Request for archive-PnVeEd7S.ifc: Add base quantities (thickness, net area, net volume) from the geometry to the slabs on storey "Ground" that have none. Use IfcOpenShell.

First a look at what the model holds.

```python
import ifcopenshell
import ifcopenshell.util.element
import ifcopenshell.util.unit

model = ifcopenshell.open("archive-PnVeEd7S.ifc")
print(model.schema)
for unit_type in ("LENGTHUNIT", "AREAUNIT", "VOLUMEUNIT"):
    print(unit_type, ifcopenshell.util.unit.calculate_unit_scale(model, unit_type))
storey = next(s for s in model.by_type("IfcBuildingStorey") if s.Name == "Ground")
slabs = [e for e in ifcopenshell.util.element.get_decomposition(storey) if e.is_a("IfcSlab")]
for e in sorted(slabs, key=lambda e: e.id()):
    print(e.id(), e.is_a(), e.Name, list(ifcopenshell.util.element.get_psets(e, qtos_only=True)), sep=" | ")
```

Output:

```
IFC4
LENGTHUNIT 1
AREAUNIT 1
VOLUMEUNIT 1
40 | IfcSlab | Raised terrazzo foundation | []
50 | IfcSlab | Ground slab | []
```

```python
import ifcopenshell
import ifcopenshell.api.pset
import ifcopenshell.geom
import ifcopenshell.util.element
import ifcopenshell.util.shape
import ifcopenshell.util.unit

model = ifcopenshell.open("archive-PnVeEd7S.ifc")
unit_scale = ifcopenshell.util.unit.calculate_unit_scale(model)
area_scale = ifcopenshell.util.unit.calculate_unit_scale(model, "AREAUNIT")
volume_scale = ifcopenshell.util.unit.calculate_unit_scale(model, "VOLUMEUNIT")
settings = ifcopenshell.geom.settings()

storey = next(s for s in model.by_type("IfcBuildingStorey") if s.Name == "Ground")
slabs = [e for e in ifcopenshell.util.element.get_decomposition(storey) if e.is_a("IfcSlab")]

for e in sorted(slabs, key=lambda e: e.id()):
    if ifcopenshell.util.element.get_psets(e, qtos_only=True, should_inherit=False):
        continue
    # Geometry comes back in metres, in the element's own axes.
    shape = ifcopenshell.geom.create_shape(settings, e)
    values = {
        "Width": ifcopenshell.util.shape.get_z(shape.geometry) / unit_scale,
        "NetArea": ifcopenshell.util.shape.get_footprint_area(shape.geometry) / area_scale,
        "NetVolume": ifcopenshell.util.shape.get_volume(shape.geometry) / volume_scale,
    }
    qto = ifcopenshell.api.pset.add_qto(model, product=e, name="Qto_SlabBaseQuantities")
    ifcopenshell.api.pset.edit_qto(model, qto=qto, properties=values)
    print(e.id(), {k: round(v, 3) for k, v in values.items()})

model.write("archive-PnVeEd7S_edited.ifc")
```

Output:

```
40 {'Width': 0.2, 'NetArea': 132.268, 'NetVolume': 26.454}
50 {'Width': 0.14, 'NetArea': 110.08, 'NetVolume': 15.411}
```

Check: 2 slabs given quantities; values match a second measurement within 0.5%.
